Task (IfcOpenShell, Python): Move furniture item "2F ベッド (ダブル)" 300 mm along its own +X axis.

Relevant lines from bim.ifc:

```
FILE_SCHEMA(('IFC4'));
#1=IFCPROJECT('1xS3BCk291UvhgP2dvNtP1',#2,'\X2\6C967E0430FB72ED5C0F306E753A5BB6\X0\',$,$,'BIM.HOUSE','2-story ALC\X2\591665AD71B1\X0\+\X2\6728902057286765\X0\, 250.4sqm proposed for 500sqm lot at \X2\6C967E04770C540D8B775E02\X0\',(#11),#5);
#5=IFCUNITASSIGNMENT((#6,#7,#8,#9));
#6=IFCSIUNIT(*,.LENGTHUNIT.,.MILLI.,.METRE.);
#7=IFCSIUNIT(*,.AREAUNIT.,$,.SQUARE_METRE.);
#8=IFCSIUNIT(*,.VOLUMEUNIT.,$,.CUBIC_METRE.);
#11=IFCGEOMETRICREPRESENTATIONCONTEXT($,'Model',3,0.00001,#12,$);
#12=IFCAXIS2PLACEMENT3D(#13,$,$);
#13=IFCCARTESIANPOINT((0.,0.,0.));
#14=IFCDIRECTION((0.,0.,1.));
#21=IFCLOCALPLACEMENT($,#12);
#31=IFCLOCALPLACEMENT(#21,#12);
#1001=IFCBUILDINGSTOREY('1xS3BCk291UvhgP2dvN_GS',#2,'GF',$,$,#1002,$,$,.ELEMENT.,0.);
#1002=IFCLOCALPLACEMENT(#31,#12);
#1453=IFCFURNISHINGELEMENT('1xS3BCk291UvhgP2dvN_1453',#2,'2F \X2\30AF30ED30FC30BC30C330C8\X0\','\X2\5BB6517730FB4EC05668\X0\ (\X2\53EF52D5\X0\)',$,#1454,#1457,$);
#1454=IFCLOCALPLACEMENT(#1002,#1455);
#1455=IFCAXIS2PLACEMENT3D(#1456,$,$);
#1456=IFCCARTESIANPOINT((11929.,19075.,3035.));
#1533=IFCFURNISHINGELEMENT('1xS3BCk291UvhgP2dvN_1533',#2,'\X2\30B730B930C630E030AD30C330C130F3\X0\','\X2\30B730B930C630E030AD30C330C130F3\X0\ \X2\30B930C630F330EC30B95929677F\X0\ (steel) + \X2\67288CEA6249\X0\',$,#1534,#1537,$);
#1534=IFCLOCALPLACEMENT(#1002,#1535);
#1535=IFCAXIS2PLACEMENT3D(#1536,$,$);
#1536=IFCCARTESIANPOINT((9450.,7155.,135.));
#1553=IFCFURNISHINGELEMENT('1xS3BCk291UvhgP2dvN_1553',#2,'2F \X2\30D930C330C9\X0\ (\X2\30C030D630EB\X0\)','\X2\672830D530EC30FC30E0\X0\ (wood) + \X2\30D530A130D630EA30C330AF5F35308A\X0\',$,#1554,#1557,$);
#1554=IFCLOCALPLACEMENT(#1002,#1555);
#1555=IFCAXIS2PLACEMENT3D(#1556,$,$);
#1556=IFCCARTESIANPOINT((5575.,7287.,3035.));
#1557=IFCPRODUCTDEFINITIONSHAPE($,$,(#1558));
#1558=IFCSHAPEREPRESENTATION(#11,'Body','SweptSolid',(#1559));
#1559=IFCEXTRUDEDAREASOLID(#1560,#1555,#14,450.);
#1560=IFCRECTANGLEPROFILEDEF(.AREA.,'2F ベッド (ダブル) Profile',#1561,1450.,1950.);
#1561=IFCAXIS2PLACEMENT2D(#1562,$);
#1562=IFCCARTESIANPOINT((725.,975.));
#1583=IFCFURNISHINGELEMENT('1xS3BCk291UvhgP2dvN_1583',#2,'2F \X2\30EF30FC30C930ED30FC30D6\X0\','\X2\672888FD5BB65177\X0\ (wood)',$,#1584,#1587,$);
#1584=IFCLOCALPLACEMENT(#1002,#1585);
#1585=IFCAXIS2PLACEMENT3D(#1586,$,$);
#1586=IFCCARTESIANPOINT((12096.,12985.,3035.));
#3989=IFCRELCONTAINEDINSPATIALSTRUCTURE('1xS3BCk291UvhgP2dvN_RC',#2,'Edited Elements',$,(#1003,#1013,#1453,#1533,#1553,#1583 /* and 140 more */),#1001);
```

```python
import ifcopenshell
import ifcopenshell.api.geometry
import ifcopenshell.util.placement
import ifcopenshell.util.unit

model = ifcopenshell.open("bim.ifc")
unit_scale = ifcopenshell.util.unit.calculate_unit_scale(model)

item = model.by_guid("1xS3BCk291UvhgP2dvN_1553")
matrix = ifcopenshell.util.placement.get_local_placement(item.ObjectPlacement)
matrix[:3, 3] += matrix[:3, 0] * 0.3 / unit_scale
ifcopenshell.api.geometry.edit_object_placement(model, product=item, matrix=matrix, is_si=False)

print(ifcopenshell.util.placement.get_local_placement(item.ObjectPlacement).round(3) + 0.0)

model.write("bim_v2.ifc")
```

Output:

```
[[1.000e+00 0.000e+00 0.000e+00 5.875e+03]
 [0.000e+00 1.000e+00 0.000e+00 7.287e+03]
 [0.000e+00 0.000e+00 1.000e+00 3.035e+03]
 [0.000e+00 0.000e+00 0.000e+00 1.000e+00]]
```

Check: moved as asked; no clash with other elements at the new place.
